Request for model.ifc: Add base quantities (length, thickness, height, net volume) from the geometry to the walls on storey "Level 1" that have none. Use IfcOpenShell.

First a look at what the model holds.

```python
import ifcopenshell
import ifcopenshell.util.element
import ifcopenshell.util.unit

model = ifcopenshell.open("model.ifc")
print(model.schema)
for unit_type in ("LENGTHUNIT", "AREAUNIT", "VOLUMEUNIT"):
    print(unit_type, ifcopenshell.util.unit.calculate_unit_scale(model, unit_type))
storey = next(s for s in model.by_type("IfcBuildingStorey") if s.Name == "Level 1")
walls = [e for e in ifcopenshell.util.element.get_decomposition(storey) if e.is_a("IfcWall")]
for e in sorted(walls, key=lambda e: e.id()):
    print(e.id(), e.is_a(), e.Name, list(ifcopenshell.util.element.get_psets(e, qtos_only=True)), sep=" | ")
```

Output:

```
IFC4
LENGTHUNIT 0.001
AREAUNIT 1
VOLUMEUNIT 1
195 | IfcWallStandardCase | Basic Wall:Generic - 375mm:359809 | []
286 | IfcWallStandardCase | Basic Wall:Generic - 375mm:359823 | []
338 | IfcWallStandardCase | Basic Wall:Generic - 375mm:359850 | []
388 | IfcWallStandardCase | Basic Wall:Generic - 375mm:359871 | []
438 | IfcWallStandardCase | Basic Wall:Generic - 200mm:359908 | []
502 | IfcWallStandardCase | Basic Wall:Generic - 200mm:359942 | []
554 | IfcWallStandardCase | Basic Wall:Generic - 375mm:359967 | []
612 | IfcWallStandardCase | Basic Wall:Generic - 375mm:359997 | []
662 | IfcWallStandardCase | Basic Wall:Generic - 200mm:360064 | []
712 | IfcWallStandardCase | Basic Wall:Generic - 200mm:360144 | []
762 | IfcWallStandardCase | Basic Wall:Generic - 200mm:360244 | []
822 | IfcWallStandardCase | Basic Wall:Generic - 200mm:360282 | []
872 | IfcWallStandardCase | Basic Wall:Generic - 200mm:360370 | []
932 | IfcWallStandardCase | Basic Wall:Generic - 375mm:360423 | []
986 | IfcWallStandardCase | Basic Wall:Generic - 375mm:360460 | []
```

```python
import ifcopenshell
import ifcopenshell.api.pset
import ifcopenshell.geom
import ifcopenshell.util.element
import ifcopenshell.util.shape
import ifcopenshell.util.unit

model = ifcopenshell.open("model.ifc")
unit_scale = ifcopenshell.util.unit.calculate_unit_scale(model)
volume_scale = ifcopenshell.util.unit.calculate_unit_scale(model, "VOLUMEUNIT")
settings = ifcopenshell.geom.settings()

storey = next(s for s in model.by_type("IfcBuildingStorey") if s.Name == "Level 1")
walls = [e for e in ifcopenshell.util.element.get_decomposition(storey) if e.is_a("IfcWall")]

for e in sorted(walls, key=lambda e: e.id()):
    if ifcopenshell.util.element.get_psets(e, qtos_only=True, should_inherit=False):
        continue
    # Geometry comes back in metres, in the element's own axes.
    shape = ifcopenshell.geom.create_shape(settings, e)
    values = {
        "Length": ifcopenshell.util.shape.get_x(shape.geometry) / unit_scale,
        "Width": ifcopenshell.util.shape.get_y(shape.geometry) / unit_scale,
        "Height": ifcopenshell.util.shape.get_z(shape.geometry) / unit_scale,
        "NetVolume": ifcopenshell.util.shape.get_volume(shape.geometry) / volume_scale,
    }
    qto = ifcopenshell.api.pset.add_qto(model, product=e, name="Qto_WallBaseQuantities")
    ifcopenshell.api.pset.edit_qto(model, qto=qto, properties=values)
    print(e.id(), {k: round(v, 3) for k, v in values.items()})

model.write("model_edited.ifc")
```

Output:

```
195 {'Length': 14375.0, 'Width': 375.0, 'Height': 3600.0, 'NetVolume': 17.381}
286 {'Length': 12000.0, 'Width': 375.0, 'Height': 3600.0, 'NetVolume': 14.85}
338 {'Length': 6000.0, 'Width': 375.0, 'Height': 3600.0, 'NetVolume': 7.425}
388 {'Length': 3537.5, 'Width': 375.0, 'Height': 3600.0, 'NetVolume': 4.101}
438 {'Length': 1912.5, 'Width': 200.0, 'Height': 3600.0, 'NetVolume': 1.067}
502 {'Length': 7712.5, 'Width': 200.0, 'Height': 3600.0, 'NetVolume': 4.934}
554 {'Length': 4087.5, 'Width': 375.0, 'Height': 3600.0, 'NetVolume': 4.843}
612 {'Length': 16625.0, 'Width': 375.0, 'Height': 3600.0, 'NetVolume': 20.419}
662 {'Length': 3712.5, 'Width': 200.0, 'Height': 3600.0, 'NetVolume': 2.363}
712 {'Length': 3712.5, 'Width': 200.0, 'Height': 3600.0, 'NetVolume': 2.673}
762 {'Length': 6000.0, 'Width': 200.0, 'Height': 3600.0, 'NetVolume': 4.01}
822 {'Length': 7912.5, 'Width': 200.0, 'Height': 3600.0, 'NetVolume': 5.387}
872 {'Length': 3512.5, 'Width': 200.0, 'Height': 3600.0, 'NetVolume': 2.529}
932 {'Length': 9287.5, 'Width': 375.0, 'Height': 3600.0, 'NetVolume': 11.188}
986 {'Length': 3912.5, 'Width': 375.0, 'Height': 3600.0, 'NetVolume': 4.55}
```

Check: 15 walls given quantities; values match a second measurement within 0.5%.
